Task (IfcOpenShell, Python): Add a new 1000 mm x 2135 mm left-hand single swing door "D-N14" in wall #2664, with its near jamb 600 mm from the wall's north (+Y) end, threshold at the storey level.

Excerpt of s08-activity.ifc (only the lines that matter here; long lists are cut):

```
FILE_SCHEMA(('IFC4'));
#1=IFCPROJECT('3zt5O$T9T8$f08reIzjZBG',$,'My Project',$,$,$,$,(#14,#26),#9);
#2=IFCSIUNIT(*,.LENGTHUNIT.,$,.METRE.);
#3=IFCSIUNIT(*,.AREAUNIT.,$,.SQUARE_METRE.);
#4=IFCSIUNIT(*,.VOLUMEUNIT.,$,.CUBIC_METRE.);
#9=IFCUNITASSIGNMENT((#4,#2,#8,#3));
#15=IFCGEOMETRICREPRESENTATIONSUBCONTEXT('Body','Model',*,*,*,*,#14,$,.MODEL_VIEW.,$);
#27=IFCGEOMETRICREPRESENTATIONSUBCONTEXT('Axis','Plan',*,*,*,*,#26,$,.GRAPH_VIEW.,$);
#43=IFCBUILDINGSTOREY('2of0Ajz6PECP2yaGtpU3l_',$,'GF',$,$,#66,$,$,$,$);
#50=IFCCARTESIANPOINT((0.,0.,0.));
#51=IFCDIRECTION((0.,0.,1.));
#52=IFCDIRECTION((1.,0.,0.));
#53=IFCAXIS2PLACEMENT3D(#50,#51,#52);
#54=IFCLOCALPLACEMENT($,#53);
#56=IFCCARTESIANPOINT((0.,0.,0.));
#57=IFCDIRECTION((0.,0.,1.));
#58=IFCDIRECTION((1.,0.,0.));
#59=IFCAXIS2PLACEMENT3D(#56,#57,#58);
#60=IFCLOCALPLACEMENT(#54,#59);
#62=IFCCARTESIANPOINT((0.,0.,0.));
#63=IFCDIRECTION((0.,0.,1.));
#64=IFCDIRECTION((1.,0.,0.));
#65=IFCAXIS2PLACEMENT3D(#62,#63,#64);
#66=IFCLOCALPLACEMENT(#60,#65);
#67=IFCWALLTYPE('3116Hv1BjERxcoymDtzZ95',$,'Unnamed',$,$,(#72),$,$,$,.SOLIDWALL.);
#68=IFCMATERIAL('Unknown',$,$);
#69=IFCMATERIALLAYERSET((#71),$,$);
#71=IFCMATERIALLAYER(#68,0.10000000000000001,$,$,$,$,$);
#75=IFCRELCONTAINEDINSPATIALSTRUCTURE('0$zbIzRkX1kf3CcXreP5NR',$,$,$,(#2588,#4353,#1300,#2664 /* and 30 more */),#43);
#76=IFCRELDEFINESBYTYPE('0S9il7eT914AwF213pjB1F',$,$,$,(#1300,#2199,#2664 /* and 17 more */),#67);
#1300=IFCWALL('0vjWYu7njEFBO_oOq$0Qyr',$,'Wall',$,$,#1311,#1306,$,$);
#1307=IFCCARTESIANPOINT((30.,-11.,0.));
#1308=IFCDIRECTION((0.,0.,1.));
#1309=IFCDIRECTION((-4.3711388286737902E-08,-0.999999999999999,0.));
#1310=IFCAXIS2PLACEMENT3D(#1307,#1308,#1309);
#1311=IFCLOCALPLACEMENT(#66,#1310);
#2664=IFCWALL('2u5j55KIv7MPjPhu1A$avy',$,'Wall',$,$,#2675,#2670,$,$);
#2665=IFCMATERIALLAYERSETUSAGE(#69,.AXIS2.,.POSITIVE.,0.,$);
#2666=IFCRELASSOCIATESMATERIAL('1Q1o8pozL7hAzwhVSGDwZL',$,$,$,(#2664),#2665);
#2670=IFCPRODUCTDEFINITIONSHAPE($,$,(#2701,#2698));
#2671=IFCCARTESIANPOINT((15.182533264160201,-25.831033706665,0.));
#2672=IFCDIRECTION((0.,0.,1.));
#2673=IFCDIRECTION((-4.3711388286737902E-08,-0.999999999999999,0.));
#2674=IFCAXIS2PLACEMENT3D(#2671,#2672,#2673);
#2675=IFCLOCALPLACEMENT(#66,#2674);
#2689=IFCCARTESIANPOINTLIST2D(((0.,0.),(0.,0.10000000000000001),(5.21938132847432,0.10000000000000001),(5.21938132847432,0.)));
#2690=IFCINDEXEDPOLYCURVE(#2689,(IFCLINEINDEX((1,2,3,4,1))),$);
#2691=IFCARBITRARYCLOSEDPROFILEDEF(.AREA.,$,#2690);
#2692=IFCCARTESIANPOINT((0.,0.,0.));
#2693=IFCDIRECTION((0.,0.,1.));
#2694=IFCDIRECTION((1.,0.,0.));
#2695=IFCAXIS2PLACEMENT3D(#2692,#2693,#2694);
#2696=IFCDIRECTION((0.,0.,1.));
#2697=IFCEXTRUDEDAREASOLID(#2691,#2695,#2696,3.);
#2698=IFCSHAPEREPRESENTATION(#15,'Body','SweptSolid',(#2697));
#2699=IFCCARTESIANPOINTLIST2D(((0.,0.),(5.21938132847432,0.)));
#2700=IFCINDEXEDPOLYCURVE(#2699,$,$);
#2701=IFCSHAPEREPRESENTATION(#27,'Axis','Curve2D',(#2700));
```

```python
import numpy as np
import ifcopenshell
import ifcopenshell.api.feature
import ifcopenshell.api.geometry
import ifcopenshell.api.root
import ifcopenshell.api.spatial
import ifcopenshell.geom
import ifcopenshell.util.element
import ifcopenshell.util.placement
import ifcopenshell.util.representation
import ifcopenshell.util.shape
import ifcopenshell.util.unit

model = ifcopenshell.open("s08-activity.ifc")
unit_scale = ifcopenshell.util.unit.calculate_unit_scale(model)
settings = ifcopenshell.geom.settings()


def volume(element):
    """Net volume in cubic metres, openings subtracted."""
    shape = ifcopenshell.geom.create_shape(settings, element)
    return ifcopenshell.util.shape.get_volume(shape.geometry)


wall = model.by_id(2664)
storey = ifcopenshell.util.element.get_container(wall, ifc_class="IfcBuildingStorey")
context = ifcopenshell.util.representation.get_context(model, "Model", "Body", "MODEL_VIEW")
before = volume(wall)

width, height, from_end, sill = 1, 2.135, 0.6, 0.0  # metres

# The wall runs along its own X axis, and the end named is its -X end.
wall_shape = ifcopenshell.geom.create_shape(settings, wall)
x, y, z = ifcopenshell.util.shape.get_vertices(wall_shape.geometry).T
start = x.min() + from_end
face, thickness = float(y.min()), float(y.max() - y.min())
wall_matrix = ifcopenshell.util.placement.get_local_placement(wall.ObjectPlacement)
level = ifcopenshell.util.placement.get_local_placement(storey.ObjectPlacement)[2, 3]


def in_wall(x, y):
    """Placement at x, y metres in the wall's axes, at sill height."""
    matrix = wall_matrix.copy()
    matrix[:, 3] = wall_matrix @ np.array([x / unit_scale, y / unit_scale, 0.0, 1.0])
    matrix[2, 3] = level + sill / unit_scale
    return matrix


# Opening: a box that overshoots both wall faces by 50 mm.
opening = ifcopenshell.api.root.create_entity(model, ifc_class="IfcOpeningElement", predefined_type="OPENING")
box = ifcopenshell.api.geometry.add_wall_representation(
    model, context=context, length=width, height=height, thickness=thickness + 0.1
)
ifcopenshell.api.geometry.assign_representation(model, product=opening, representation=box)
ifcopenshell.api.geometry.edit_object_placement(model, product=opening, matrix=in_wall(start, face - 0.05), is_si=False)
ifcopenshell.api.feature.add_feature(model, feature=opening, element=wall)

door = ifcopenshell.api.root.create_entity(model, ifc_class="IfcDoor", name="D-N14", predefined_type="DOOR")
door.OverallWidth, door.OverallHeight = width / unit_scale, height / unit_scale
door.OperationType = "SINGLE_SWING_LEFT"
body = ifcopenshell.api.geometry.add_door_representation(
    model,
    context=context,
    overall_width=door.OverallWidth,
    overall_height=door.OverallHeight,
    operation_type="SINGLE_SWING_LEFT",
    lining_properties={"LiningDepth": thickness / unit_scale, "ThresholdDepth": thickness / unit_scale},
)
ifcopenshell.api.geometry.assign_representation(model, product=door, representation=body)
ifcopenshell.api.spatial.assign_container(model, products=[door], relating_structure=storey)
ifcopenshell.api.feature.add_filling(model, opening=opening, element=door)

# The lining spans the wall, so the door starts at the wall face.
ifcopenshell.api.geometry.edit_object_placement(model, product=door, matrix=in_wall(start, face), is_si=False)

after = volume(wall)

print(f"wall volume {before:.3f} -> {after:.3f} m3")

model.write("s08-activity-out.ifc")
```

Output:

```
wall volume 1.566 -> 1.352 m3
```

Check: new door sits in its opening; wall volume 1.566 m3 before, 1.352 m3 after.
